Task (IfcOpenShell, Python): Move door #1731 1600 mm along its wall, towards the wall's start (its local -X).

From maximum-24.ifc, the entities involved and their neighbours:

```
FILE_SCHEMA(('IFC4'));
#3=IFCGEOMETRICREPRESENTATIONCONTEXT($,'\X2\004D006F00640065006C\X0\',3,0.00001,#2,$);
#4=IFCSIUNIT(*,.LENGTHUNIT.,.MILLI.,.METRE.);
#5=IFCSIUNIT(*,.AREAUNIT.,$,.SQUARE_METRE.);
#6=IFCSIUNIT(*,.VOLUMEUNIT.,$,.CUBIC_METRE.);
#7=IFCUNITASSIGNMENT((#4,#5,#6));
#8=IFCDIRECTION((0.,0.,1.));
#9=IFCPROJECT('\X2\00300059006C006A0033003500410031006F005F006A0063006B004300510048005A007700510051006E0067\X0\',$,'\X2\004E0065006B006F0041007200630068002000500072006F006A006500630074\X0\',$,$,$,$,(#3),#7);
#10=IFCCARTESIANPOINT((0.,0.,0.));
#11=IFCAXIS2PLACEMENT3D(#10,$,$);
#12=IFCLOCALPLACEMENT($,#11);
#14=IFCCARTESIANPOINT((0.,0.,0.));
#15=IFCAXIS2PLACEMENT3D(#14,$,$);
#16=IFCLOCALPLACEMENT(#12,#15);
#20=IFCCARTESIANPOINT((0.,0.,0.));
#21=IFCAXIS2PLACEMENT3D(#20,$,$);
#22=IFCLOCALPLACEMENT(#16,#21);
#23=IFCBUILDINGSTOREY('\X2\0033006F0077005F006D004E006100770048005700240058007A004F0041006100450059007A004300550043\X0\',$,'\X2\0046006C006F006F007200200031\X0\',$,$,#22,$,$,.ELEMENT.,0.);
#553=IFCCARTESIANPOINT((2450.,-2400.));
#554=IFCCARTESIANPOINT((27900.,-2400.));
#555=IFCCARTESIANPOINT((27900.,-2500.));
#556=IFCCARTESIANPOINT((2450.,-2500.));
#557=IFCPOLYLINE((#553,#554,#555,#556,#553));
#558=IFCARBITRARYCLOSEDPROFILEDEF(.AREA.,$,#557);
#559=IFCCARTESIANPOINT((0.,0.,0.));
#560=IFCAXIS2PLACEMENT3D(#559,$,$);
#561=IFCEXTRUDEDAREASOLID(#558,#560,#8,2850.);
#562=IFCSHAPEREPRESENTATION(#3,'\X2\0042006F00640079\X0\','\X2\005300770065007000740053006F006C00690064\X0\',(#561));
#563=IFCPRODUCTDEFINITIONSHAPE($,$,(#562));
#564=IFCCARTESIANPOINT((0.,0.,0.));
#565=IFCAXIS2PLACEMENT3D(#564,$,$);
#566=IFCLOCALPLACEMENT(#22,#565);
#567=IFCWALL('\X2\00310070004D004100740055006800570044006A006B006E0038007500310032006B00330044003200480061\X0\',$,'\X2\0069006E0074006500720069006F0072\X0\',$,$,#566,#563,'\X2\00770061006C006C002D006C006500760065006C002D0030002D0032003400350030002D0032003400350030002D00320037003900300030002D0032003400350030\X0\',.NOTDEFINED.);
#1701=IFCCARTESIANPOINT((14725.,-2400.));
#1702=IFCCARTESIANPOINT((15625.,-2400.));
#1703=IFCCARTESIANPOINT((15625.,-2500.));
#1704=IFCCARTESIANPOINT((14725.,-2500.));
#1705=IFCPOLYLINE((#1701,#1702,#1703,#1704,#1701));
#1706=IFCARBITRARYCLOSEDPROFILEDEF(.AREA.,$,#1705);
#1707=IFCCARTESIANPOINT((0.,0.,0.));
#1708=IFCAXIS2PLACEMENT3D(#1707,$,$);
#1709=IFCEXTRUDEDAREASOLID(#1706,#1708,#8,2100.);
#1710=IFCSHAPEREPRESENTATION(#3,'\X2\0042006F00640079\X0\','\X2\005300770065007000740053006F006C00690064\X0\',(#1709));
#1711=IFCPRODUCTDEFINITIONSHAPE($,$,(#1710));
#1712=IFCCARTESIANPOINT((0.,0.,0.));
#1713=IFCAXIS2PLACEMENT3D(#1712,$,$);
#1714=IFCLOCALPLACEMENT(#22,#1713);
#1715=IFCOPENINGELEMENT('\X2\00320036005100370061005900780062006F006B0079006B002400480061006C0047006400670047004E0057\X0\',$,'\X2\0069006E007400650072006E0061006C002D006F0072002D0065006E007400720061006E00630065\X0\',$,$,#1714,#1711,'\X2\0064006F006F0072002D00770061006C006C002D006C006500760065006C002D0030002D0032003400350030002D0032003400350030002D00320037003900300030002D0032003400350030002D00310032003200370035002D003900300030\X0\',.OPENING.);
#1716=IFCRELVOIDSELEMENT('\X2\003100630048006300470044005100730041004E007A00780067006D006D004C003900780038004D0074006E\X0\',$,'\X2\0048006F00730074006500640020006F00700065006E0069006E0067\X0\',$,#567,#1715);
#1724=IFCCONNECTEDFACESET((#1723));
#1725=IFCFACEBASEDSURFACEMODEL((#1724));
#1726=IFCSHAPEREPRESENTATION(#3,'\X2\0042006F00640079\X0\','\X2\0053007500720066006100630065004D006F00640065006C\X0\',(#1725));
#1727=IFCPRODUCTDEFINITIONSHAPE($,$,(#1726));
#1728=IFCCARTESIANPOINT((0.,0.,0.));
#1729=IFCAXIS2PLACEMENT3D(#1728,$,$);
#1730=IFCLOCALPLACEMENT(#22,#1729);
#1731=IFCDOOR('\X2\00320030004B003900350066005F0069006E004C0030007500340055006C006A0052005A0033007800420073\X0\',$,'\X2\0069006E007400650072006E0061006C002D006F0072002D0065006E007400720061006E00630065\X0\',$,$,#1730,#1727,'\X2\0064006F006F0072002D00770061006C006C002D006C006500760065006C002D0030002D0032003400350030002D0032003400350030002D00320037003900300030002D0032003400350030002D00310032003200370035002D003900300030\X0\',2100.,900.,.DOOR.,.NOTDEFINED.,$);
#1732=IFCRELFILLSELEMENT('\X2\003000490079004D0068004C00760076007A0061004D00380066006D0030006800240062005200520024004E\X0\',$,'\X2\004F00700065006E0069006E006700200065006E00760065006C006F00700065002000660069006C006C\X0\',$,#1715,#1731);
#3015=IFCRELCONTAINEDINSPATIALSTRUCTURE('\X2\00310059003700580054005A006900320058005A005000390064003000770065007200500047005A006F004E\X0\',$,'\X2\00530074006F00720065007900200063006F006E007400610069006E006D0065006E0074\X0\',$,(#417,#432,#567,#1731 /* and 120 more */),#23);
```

```python
import ifcopenshell
import ifcopenshell.api.geometry
import ifcopenshell.util.placement
import ifcopenshell.util.unit

model = ifcopenshell.open("maximum-24.ifc")
unit_scale = ifcopenshell.util.unit.calculate_unit_scale(model)

door = model.by_id(1731)
opening = door.FillsVoids[0].RelatingOpeningElement
wall = opening.VoidsElements[0].RelatingBuildingElement

wall_matrix = ifcopenshell.util.placement.get_local_placement(wall.ObjectPlacement)
shift = wall_matrix[:3, 0] * -1.6 / unit_scale
before = ifcopenshell.util.placement.get_local_placement(door.ObjectPlacement)[:3, 3].copy()

# The door is not placed relative to its opening, so move both.
for product in (opening, door):
    matrix = ifcopenshell.util.placement.get_local_placement(product.ObjectPlacement)
    matrix[:3, 3] += shift
    ifcopenshell.api.geometry.edit_object_placement(model, product=product, matrix=matrix, is_si=False)

after = ifcopenshell.util.placement.get_local_placement(door.ObjectPlacement)[:3, 3]
print("door moved by", (after - before).round(3) + 0.0)

model.write("maximum-24_edited.ifc")
```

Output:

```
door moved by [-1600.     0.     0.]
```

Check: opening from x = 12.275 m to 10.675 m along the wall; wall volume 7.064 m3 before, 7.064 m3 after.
